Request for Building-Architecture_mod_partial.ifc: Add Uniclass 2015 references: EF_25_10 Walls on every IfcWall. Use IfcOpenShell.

First a look at what the model holds.

```python
import ifcopenshell

model = ifcopenshell.open("Building-Architecture_mod_partial.ifc")
print(model.schema)
print("classifications:", [c.Name for c in model.by_type("IfcClassification")])
for ifc_class in ("IfcDoor", "IfcRoof", "IfcStair", "IfcWall", "IfcWindow"):
    print(ifc_class, len(model.by_type(ifc_class)))
```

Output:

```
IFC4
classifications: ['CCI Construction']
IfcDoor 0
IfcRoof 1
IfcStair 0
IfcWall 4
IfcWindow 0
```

```python
import ifcopenshell
import ifcopenshell.api.classification

model = ifcopenshell.open("Building-Architecture_mod_partial.ifc")

system = ifcopenshell.api.classification.add_classification(model, classification="Uniclass 2015")

codes = {
    "IfcWall": ("EF_25_10", "Walls"),
}
for ifc_class, (code, name) in codes.items():
    products = model.by_type(ifc_class)
    ifcopenshell.api.classification.add_reference(
        model, products=products, classification=system, identification=code, name=name
    )
    print(code, len(products))

model.write("Building-Architecture_mod_partial_rev.ifc")
```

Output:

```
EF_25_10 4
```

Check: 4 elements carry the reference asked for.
